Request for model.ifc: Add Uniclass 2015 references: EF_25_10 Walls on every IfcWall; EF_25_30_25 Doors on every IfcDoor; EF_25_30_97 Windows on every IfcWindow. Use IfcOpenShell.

First a look at what the model holds.

```python
import ifcopenshell

model = ifcopenshell.open("model.ifc")
print(model.schema)
print("classifications:", [c.Name for c in model.by_type("IfcClassification")])
for ifc_class in ("IfcDoor", "IfcRoof", "IfcStair", "IfcWall", "IfcWindow"):
    print(ifc_class, len(model.by_type(ifc_class)))
```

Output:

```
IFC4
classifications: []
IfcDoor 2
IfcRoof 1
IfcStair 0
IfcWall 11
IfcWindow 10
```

```python
import ifcopenshell
import ifcopenshell.api.classification

model = ifcopenshell.open("model.ifc")

system = ifcopenshell.api.classification.add_classification(model, classification="Uniclass 2015")

codes = {
    "IfcWall": ("EF_25_10", "Walls"),
    "IfcDoor": ("EF_25_30_25", "Doors"),
    "IfcWindow": ("EF_25_30_97", "Windows"),
}
for ifc_class, (code, name) in codes.items():
    products = model.by_type(ifc_class)
    ifcopenshell.api.classification.add_reference(
        model, products=products, classification=system, identification=code, name=name
    )
    print(code, len(products))

model.write("model_edited.ifc")
```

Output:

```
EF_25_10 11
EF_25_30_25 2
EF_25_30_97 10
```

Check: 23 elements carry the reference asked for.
